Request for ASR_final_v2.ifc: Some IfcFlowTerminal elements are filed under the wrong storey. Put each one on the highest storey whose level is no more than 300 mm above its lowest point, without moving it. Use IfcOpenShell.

First a look at what the model holds.

```python
import ifcopenshell
import ifcopenshell.util.element
import ifcopenshell.util.placement

model = ifcopenshell.open("ASR_final_v2.ifc")
print(model.schema)
for storey in model.by_type("IfcBuildingStorey"):
    level = ifcopenshell.util.placement.get_storey_elevation(storey)
    count = sum(e.is_a("IfcFlowTerminal") for e in ifcopenshell.util.element.get_contained(storey))
    print(storey.id(), storey.Name, round(level, 3), count, sep=" | ")
```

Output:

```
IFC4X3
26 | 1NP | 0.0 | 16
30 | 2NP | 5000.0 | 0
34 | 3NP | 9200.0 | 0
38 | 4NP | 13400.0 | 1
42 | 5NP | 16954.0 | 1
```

```python
import ifcopenshell
import ifcopenshell.api.spatial
import ifcopenshell.geom
import ifcopenshell.util.element
import ifcopenshell.util.placement
import ifcopenshell.util.shape
import ifcopenshell.util.unit

model = ifcopenshell.open("ASR_final_v2.ifc")
unit_scale = ifcopenshell.util.unit.calculate_unit_scale(model)
settings = ifcopenshell.geom.settings()

levels = sorted(
    ((ifcopenshell.util.placement.get_storey_elevation(s) * unit_scale, s) for s in model.by_type("IfcBuildingStorey")),
    key=lambda pair: pair[0],
)

for e in model.by_type("IfcFlowTerminal"):
    current = e.ContainedInStructure[0].RelatingStructure if e.ContainedInStructure else None
    if current is None or not current.is_a("IfcBuildingStorey"):
        continue
    shape = ifcopenshell.geom.create_shape(settings, e)
    bottom = ifcopenshell.util.shape.get_shape_bottom_elevation(shape, shape.geometry)
    below = [s for level, s in levels if level <= bottom + 0.3]
    storey = below[-1] if below else levels[0][1]
    if storey != current:
        # assign_container keeps the world position.
        ifcopenshell.api.spatial.assign_container(model, products=[e], relating_structure=storey)
        print(e.id(), current.Name, "->", storey.Name)

model.write("ASR_final_v2_rev.ifc")
```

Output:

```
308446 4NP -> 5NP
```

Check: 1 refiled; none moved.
